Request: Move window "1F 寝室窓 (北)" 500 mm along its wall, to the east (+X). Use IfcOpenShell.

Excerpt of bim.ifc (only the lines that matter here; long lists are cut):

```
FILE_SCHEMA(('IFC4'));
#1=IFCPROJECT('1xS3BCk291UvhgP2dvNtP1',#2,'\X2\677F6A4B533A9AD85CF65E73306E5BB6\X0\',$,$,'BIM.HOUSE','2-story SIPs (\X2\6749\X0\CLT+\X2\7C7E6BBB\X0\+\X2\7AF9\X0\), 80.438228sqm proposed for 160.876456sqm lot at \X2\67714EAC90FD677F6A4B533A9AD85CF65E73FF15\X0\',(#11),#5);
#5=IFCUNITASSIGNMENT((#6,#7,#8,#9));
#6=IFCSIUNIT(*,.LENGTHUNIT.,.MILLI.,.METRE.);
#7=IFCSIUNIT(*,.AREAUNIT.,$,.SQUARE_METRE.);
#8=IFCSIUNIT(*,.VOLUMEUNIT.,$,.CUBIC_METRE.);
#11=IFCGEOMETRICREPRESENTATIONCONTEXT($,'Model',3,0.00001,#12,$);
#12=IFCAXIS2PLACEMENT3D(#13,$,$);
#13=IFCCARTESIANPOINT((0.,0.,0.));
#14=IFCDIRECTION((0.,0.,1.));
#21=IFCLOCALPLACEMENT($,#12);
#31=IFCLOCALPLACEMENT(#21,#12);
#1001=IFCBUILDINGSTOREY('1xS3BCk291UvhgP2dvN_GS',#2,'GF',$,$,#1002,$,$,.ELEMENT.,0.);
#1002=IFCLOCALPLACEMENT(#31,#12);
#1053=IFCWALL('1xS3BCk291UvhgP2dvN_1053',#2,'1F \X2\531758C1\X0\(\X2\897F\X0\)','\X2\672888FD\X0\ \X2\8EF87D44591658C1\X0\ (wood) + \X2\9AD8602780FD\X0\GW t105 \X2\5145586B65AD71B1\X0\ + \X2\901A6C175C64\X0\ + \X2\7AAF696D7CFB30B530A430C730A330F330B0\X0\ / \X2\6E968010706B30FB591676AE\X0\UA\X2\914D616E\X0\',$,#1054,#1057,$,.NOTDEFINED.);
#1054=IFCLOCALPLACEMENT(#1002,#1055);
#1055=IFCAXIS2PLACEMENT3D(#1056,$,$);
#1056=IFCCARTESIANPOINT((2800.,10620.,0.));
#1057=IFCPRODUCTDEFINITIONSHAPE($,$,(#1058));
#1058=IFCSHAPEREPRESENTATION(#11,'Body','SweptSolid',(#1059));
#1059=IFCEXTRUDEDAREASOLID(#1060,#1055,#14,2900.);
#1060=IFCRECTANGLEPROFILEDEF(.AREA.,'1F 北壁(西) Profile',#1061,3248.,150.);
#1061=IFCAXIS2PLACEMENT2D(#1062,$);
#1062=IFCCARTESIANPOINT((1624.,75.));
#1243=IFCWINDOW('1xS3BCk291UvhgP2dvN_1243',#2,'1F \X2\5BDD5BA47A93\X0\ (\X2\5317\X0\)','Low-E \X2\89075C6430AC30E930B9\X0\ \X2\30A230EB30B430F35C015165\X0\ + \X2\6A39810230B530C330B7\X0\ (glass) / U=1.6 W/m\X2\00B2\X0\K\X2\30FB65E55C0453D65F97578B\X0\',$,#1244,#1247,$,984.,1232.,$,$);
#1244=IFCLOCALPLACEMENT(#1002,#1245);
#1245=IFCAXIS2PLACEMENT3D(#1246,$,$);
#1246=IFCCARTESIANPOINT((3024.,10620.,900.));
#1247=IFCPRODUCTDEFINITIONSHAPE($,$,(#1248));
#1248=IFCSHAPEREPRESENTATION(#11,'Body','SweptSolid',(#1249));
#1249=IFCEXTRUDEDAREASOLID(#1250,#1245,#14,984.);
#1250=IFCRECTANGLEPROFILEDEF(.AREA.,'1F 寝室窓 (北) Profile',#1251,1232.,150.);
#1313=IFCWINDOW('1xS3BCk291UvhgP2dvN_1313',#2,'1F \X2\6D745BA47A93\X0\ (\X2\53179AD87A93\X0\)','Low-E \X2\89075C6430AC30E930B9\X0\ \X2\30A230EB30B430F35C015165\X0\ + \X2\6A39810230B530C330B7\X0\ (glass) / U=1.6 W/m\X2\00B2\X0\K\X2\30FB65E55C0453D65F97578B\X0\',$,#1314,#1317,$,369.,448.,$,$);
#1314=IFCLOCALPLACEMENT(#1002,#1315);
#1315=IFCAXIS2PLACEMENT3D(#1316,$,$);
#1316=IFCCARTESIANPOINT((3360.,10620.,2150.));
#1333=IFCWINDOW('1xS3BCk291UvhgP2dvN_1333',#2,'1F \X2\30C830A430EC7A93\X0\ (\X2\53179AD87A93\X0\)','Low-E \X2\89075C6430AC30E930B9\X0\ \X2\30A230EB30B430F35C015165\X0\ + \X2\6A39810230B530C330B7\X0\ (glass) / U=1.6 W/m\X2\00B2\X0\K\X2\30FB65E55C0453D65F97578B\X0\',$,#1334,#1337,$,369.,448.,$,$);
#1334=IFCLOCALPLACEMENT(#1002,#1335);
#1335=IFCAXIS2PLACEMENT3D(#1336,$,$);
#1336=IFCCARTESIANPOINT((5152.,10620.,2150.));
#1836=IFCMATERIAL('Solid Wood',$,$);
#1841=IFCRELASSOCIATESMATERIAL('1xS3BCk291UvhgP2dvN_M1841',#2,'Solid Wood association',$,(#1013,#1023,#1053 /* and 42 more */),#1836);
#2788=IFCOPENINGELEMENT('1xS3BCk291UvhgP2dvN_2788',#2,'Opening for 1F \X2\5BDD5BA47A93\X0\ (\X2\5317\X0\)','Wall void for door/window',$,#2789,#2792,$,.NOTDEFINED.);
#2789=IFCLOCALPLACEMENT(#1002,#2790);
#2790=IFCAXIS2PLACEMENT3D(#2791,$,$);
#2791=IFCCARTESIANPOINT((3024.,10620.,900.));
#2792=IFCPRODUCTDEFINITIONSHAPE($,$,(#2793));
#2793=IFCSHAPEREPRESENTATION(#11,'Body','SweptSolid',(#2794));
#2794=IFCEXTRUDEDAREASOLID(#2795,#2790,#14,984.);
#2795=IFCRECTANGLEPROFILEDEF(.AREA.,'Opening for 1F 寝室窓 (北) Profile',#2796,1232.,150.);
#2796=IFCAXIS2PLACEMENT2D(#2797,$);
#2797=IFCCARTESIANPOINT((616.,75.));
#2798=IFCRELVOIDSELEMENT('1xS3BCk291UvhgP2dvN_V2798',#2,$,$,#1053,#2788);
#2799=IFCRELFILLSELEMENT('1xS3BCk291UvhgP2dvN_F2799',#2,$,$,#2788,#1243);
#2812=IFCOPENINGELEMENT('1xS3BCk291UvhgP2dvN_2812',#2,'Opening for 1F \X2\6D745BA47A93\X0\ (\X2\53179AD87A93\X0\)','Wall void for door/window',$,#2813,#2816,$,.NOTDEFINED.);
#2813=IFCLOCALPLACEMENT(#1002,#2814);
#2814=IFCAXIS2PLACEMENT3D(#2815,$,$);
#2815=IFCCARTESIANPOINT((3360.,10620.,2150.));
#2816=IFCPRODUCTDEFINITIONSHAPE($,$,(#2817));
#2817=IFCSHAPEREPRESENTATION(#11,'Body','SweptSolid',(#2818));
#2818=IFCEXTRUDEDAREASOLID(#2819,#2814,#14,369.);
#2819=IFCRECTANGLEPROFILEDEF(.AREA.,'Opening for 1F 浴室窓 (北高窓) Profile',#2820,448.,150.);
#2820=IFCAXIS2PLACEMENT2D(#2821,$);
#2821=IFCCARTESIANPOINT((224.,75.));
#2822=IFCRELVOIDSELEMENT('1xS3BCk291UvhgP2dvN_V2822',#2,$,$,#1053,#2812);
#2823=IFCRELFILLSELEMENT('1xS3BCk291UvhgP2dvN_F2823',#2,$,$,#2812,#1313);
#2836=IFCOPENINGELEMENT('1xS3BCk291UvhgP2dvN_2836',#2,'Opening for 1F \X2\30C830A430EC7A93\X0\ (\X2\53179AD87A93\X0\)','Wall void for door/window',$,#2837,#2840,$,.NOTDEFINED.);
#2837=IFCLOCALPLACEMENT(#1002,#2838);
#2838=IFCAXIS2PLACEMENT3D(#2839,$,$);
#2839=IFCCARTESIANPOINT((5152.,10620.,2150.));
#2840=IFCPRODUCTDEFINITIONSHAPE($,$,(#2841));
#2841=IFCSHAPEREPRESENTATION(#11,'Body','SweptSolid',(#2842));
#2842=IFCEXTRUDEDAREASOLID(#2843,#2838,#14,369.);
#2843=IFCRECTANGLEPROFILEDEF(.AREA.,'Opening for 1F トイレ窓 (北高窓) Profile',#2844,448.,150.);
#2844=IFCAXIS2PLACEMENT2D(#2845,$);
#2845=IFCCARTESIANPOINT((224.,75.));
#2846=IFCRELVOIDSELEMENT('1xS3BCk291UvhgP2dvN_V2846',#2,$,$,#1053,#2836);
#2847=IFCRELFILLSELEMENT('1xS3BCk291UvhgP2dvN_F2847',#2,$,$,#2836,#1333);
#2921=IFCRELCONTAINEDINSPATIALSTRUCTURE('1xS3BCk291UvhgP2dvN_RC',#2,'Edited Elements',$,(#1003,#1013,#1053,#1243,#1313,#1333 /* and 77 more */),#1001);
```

```python
import ifcopenshell
import ifcopenshell.api.geometry
import ifcopenshell.util.placement

model = ifcopenshell.open("bim.ifc")

window = model.by_guid("1xS3BCk291UvhgP2dvN_1243")
opening = window.FillsVoids[0].RelatingOpeningElement
wall = opening.VoidsElements[0].RelatingBuildingElement

wall_matrix = ifcopenshell.util.placement.get_local_placement(wall.ObjectPlacement)
shift = wall_matrix[:3, 0] * 500.0
before = ifcopenshell.util.placement.get_local_placement(window.ObjectPlacement)[:3, 3].copy()

# The window is not placed relative to its opening, so move both.
for product in (opening, window):
    matrix = ifcopenshell.util.placement.get_local_placement(product.ObjectPlacement)
    matrix[:3, 3] += shift
    ifcopenshell.api.geometry.edit_object_placement(model, product=product, matrix=matrix, is_si=False)

after = ifcopenshell.util.placement.get_local_placement(window.ObjectPlacement)[:3, 3]
print("window moved by", (after - before).round(3) + 0.0)

model.write("bim-out.ifc")
```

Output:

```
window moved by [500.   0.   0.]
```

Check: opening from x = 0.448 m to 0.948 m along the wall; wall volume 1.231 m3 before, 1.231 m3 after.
